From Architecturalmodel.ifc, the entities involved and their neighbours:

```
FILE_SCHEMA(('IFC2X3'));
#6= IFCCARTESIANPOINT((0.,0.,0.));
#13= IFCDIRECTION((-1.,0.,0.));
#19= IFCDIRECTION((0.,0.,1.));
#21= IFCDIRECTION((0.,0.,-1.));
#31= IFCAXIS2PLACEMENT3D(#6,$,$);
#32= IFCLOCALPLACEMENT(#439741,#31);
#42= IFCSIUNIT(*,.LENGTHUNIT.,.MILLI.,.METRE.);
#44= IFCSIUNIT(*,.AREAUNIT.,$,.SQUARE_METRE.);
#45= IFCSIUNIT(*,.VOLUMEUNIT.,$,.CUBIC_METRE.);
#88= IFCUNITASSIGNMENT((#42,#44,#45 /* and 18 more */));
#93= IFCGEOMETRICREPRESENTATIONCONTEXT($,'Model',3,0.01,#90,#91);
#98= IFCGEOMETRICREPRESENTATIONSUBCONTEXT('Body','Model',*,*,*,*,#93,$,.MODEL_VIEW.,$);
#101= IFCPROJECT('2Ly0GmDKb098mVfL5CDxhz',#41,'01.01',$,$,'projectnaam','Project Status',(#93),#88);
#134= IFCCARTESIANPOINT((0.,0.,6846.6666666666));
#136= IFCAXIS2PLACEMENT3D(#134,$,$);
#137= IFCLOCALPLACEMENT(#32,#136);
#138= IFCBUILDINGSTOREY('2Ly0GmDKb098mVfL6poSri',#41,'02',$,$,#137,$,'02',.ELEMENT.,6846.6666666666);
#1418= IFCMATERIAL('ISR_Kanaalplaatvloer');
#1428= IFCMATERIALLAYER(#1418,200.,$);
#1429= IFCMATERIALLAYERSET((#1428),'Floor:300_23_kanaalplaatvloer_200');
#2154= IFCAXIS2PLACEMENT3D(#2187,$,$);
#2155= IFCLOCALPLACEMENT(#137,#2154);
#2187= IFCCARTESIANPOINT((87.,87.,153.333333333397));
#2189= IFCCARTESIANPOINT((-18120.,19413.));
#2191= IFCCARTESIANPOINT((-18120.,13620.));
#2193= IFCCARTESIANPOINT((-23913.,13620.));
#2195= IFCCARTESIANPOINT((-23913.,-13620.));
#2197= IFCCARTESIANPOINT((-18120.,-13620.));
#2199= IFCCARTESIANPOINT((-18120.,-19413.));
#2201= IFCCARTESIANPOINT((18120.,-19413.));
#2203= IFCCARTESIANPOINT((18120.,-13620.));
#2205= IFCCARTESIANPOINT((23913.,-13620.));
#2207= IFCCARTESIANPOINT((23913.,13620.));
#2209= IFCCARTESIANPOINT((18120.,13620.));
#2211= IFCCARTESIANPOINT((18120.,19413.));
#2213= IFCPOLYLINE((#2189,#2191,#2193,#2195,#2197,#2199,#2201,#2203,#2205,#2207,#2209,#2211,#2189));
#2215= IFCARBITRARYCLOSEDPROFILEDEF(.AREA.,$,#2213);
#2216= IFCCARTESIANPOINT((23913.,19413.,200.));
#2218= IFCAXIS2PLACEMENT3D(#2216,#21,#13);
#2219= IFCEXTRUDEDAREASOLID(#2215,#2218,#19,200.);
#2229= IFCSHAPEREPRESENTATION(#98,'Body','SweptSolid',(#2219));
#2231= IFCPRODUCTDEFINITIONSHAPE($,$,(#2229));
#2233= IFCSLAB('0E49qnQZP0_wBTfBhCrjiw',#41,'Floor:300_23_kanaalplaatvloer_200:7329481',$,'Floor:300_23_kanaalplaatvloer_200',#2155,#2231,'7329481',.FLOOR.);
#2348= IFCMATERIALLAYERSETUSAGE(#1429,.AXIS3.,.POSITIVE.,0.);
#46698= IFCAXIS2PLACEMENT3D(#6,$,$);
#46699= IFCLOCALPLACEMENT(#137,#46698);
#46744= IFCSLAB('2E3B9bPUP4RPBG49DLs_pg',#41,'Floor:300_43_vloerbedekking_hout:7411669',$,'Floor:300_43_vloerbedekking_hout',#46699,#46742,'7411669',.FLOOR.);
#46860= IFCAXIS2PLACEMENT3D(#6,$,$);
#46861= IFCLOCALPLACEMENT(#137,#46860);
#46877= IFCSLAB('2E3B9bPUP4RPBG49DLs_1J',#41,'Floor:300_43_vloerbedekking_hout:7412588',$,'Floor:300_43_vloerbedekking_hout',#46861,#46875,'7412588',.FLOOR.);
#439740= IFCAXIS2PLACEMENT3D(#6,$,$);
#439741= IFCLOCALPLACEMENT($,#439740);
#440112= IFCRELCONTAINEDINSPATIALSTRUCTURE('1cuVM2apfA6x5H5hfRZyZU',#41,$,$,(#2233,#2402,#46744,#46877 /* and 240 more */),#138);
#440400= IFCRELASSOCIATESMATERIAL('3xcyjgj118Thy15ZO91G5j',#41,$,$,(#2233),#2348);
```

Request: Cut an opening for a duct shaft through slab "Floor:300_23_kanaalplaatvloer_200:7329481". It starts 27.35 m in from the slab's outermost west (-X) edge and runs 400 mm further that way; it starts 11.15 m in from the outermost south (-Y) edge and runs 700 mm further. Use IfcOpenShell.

```python
import numpy as np
import ifcopenshell
import ifcopenshell.api.feature
import ifcopenshell.api.geometry
import ifcopenshell.api.root
import ifcopenshell.geom
import ifcopenshell.util.placement
import ifcopenshell.util.representation
import ifcopenshell.util.shape
import ifcopenshell.util.unit

model = ifcopenshell.open("Architecturalmodel.ifc")
unit_scale = ifcopenshell.util.unit.calculate_unit_scale(model)
settings = ifcopenshell.geom.settings()


def volume(element):
    """Net volume in cubic metres, openings subtracted."""
    shape = ifcopenshell.geom.create_shape(settings, element)
    return ifcopenshell.util.shape.get_volume(shape.geometry)


slab = model.by_guid("0E49qnQZP0_wBTfBhCrjiw")
before = volume(slab)

# Extent in the slab's own axes, in metres. The edges named are its -X and -Y sides.
slab_shape = ifcopenshell.geom.create_shape(settings, slab)
vertices = ifcopenshell.util.shape.get_vertices(slab_shape.geometry)
x_min, y_min, bottom = vertices.min(axis=0)
top = vertices[:, 2].max()

opening = ifcopenshell.api.root.create_entity(model, ifc_class="IfcOpeningElement", name="Duct shaft opening")
context = ifcopenshell.util.representation.get_context(model, "Model", "Body", "MODEL_VIEW")
width, depth = 0.4, 0.7
outline = [(0.0, 0.0), (width, 0.0), (width, depth), (0.0, depth), (0.0, 0.0)]
# Overshoot both faces by 50 mm so the cut is clean.
shape = ifcopenshell.api.geometry.add_slab_representation(
    model, context=context, depth=top - bottom + 0.1, polyline=outline
)
ifcopenshell.api.geometry.assign_representation(model, product=opening, representation=shape)

matrix = ifcopenshell.util.placement.get_local_placement(slab.ObjectPlacement)
matrix[:, 3] = matrix @ np.append(np.array([x_min + 27.35, y_min + 11.15, bottom - 0.05]) / unit_scale, 1.0)
ifcopenshell.api.geometry.edit_object_placement(model, product=opening, matrix=matrix, is_si=False)
ifcopenshell.api.feature.add_feature(model, feature=opening, element=slab)

after = volume(slab)

print(f"slab volume {before:.3f} -> {after:.3f} m3")

model.write("Architecturalmodel_edited.ifc")
```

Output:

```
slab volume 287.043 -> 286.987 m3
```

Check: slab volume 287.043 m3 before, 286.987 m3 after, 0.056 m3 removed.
